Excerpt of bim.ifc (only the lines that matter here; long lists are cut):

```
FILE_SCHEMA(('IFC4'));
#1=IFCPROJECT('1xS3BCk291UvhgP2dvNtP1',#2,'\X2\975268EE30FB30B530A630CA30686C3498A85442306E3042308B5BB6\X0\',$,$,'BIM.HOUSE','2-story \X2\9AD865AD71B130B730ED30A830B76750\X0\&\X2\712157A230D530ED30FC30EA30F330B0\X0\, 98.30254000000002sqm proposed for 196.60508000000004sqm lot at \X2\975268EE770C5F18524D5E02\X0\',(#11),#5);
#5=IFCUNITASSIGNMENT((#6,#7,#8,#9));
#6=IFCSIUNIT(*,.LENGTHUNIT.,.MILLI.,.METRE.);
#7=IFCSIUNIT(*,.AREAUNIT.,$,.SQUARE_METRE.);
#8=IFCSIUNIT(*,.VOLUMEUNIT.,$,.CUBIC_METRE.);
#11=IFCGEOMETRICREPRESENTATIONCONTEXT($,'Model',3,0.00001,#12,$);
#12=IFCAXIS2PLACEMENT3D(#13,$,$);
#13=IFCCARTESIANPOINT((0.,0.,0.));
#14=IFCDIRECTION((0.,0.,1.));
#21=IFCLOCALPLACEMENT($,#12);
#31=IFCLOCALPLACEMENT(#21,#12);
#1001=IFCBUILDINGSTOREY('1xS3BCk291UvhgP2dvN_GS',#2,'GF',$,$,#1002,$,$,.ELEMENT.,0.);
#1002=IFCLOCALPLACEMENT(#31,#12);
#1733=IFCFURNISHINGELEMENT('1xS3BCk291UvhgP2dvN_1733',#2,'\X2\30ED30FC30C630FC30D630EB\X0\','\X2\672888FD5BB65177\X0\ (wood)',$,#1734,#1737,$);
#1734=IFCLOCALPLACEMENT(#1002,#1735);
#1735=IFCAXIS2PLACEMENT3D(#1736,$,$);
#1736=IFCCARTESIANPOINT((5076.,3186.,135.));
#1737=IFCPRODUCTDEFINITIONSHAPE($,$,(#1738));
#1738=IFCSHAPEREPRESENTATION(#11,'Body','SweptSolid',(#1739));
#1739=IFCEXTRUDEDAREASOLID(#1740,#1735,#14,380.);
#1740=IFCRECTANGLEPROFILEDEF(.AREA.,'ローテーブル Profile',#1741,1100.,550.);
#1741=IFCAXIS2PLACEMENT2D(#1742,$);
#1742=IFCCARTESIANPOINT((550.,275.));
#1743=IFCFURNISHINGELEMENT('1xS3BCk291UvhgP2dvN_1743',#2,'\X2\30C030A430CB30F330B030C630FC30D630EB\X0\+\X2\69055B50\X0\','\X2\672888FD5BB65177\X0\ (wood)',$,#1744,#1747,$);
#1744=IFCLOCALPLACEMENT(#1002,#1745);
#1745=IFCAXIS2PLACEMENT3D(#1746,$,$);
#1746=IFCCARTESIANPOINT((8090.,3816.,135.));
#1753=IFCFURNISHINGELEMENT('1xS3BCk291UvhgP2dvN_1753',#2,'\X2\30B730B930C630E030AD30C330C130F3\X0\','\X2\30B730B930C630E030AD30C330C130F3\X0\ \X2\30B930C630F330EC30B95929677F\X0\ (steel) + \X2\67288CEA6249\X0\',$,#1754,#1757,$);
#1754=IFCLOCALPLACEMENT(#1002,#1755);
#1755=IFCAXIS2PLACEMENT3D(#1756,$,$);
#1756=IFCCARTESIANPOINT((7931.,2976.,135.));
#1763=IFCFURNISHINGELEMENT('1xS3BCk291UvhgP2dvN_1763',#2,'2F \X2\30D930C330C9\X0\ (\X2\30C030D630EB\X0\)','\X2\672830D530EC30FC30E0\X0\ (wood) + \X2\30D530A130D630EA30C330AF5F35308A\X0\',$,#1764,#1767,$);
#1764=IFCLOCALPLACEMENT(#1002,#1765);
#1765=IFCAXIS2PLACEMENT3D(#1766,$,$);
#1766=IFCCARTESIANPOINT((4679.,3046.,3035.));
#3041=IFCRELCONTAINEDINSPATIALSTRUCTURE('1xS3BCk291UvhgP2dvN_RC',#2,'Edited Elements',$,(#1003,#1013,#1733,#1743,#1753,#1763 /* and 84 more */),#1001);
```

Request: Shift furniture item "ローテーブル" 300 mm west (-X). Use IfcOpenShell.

```python
import ifcopenshell
import ifcopenshell.api.geometry
import ifcopenshell.util.placement

model = ifcopenshell.open("bim.ifc")

item = model.by_guid("1xS3BCk291UvhgP2dvN_1733")
matrix = ifcopenshell.util.placement.get_local_placement(item.ObjectPlacement)
matrix[0, 3] -= 300.0
ifcopenshell.api.geometry.edit_object_placement(model, product=item, matrix=matrix, is_si=False)

print(ifcopenshell.util.placement.get_local_placement(item.ObjectPlacement).round(3) + 0.0)

model.write("bim-out.ifc")
```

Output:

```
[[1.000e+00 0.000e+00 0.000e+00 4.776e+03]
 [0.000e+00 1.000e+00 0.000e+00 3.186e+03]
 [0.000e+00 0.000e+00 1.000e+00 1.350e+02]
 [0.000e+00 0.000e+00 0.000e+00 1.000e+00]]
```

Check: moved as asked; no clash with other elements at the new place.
